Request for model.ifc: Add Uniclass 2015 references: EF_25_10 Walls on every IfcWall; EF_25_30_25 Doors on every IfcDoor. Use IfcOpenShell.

First a look at what the model holds.

```python
import ifcopenshell

model = ifcopenshell.open("model.ifc")
print(model.schema)
print("classifications:", [c.Name for c in model.by_type("IfcClassification")])
for ifc_class in ("IfcDoor", "IfcRoof", "IfcStair", "IfcWall", "IfcWindow"):
    print(ifc_class, len(model.by_type(ifc_class)))
```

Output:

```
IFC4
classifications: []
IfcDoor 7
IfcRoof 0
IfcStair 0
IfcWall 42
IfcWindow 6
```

```python
import ifcopenshell
import ifcopenshell.api.classification

model = ifcopenshell.open("model.ifc")

system = ifcopenshell.api.classification.add_classification(model, classification="Uniclass 2015")

codes = {
    "IfcWall": ("EF_25_10", "Walls"),
    "IfcDoor": ("EF_25_30_25", "Doors"),
}
for ifc_class, (code, name) in codes.items():
    products = model.by_type(ifc_class)
    ifcopenshell.api.classification.add_reference(
        model, products=products, classification=system, identification=code, name=name
    )
    print(code, len(products))

model.write("model_edited.ifc")
```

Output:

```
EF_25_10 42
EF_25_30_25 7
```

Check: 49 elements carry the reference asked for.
